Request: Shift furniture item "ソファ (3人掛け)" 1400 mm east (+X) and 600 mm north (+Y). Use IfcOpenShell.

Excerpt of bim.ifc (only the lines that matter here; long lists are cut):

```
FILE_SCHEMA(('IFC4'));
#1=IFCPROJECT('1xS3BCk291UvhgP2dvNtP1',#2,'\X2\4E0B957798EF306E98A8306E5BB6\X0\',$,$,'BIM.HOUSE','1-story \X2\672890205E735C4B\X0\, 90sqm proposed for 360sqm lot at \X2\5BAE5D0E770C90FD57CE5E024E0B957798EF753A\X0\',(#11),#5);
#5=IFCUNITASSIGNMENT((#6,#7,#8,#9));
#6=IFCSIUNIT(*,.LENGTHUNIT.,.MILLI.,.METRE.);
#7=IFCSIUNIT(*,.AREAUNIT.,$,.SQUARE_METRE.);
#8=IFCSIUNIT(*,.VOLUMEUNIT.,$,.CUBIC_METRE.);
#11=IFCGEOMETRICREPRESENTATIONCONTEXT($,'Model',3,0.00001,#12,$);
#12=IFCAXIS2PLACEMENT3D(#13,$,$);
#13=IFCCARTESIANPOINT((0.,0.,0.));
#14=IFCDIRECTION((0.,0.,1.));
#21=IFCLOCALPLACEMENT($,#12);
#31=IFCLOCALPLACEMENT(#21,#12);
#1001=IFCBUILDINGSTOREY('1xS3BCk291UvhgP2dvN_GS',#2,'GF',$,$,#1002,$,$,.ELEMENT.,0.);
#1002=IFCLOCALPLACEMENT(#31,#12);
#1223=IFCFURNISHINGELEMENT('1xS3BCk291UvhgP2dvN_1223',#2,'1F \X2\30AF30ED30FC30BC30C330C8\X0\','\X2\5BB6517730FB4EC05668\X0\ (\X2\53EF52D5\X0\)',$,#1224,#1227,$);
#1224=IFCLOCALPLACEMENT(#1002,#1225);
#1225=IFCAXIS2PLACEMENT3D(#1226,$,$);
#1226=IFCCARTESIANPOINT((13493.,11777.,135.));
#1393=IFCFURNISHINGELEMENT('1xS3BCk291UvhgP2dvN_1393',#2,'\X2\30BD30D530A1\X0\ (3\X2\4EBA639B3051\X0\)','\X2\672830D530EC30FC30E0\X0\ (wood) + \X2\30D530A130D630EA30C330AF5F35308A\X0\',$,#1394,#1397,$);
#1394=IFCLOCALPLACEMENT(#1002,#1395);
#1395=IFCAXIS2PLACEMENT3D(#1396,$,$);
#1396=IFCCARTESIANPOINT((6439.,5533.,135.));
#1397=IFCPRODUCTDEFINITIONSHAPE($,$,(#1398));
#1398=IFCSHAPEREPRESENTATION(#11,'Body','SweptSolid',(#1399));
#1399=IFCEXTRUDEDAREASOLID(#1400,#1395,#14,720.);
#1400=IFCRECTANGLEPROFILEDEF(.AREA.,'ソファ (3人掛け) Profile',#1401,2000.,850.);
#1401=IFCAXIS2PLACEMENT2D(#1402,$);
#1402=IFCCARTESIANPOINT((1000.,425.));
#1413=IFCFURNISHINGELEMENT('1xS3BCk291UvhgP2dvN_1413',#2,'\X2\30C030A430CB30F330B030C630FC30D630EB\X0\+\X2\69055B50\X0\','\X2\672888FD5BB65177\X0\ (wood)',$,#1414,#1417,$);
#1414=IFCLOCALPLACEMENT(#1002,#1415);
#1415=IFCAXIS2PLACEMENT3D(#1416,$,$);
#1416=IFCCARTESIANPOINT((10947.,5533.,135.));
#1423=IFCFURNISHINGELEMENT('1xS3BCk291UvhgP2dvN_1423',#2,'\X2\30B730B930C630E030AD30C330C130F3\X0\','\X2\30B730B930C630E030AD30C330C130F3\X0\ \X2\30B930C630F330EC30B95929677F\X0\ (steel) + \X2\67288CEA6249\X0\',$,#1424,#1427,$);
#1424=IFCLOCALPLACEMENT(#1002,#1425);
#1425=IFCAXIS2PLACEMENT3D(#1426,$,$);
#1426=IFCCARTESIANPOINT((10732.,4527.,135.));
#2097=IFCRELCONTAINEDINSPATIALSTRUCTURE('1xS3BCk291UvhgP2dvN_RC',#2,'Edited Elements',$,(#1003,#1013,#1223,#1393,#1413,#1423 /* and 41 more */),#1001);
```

```python
import ifcopenshell
import ifcopenshell.api.geometry
import ifcopenshell.util.placement
import ifcopenshell.util.unit

model = ifcopenshell.open("bim.ifc")
unit_scale = ifcopenshell.util.unit.calculate_unit_scale(model)

item = model.by_id(1393)
matrix = ifcopenshell.util.placement.get_local_placement(item.ObjectPlacement)
matrix[0, 3] += 1.4 / unit_scale
matrix[1, 3] += 0.6 / unit_scale
ifcopenshell.api.geometry.edit_object_placement(model, product=item, matrix=matrix, is_si=False)

print(ifcopenshell.util.placement.get_local_placement(item.ObjectPlacement).round(3) + 0.0)

model.write("bim_v2.ifc")
```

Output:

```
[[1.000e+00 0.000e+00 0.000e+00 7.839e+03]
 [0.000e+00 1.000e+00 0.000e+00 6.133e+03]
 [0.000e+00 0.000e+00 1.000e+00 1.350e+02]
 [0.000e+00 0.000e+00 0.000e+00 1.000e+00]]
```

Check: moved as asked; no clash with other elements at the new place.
